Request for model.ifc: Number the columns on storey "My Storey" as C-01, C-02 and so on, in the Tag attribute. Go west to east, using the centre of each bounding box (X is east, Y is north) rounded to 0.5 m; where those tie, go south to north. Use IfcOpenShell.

First a look at what the model holds.

```python
import ifcopenshell
import ifcopenshell.util.element
import ifcopenshell.util.placement

model = ifcopenshell.open("model.ifc")
print(model.schema)
storey = next(s for s in model.by_type("IfcBuildingStorey") if s.Name == "My Storey")
columns = [e for e in ifcopenshell.util.element.get_decomposition(storey) if e.is_a("IfcColumn")]
for e in sorted(columns, key=lambda e: e.id()):
    origin = ifcopenshell.util.placement.get_local_placement(e.ObjectPlacement)[:3, 3]
    print(e.id(), e.Tag, e.Name, origin.round(2) + 0.0, sep=" | ")
```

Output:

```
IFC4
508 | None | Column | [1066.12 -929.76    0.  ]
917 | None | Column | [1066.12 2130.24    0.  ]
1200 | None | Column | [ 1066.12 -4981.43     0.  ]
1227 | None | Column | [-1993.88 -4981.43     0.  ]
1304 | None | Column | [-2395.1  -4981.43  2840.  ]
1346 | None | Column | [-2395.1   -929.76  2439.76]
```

```python
import ifcopenshell
import ifcopenshell.geom
import ifcopenshell.util.element
import ifcopenshell.util.shape

model = ifcopenshell.open("model.ifc")
settings = ifcopenshell.geom.settings()
settings.set("use-world-coords", True)


def centre(element):
    shape = ifcopenshell.geom.create_shape(settings, element)
    return ifcopenshell.util.shape.get_bbox_centroid(shape.geometry)


storey = next(s for s in model.by_type("IfcBuildingStorey") if s.Name == "My Storey")
columns = [e for e in ifcopenshell.util.element.get_decomposition(storey) if e.is_a("IfcColumn")]

# Insertion points can sit at a corner or the storey origin, so sort by the geometry (in metres).
centres = {e: centre(e) for e in columns}
columns.sort(key=lambda e: (round(centres[e][0] / 0.5), centres[e][1]))

for i, e in enumerate(columns, start=1):
    number = f"C-{i:02d}"
    e.Tag = number
    print(e.id(), number)

model.write("model_v2.ifc")
```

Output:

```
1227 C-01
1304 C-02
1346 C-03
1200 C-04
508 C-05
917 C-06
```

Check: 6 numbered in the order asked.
